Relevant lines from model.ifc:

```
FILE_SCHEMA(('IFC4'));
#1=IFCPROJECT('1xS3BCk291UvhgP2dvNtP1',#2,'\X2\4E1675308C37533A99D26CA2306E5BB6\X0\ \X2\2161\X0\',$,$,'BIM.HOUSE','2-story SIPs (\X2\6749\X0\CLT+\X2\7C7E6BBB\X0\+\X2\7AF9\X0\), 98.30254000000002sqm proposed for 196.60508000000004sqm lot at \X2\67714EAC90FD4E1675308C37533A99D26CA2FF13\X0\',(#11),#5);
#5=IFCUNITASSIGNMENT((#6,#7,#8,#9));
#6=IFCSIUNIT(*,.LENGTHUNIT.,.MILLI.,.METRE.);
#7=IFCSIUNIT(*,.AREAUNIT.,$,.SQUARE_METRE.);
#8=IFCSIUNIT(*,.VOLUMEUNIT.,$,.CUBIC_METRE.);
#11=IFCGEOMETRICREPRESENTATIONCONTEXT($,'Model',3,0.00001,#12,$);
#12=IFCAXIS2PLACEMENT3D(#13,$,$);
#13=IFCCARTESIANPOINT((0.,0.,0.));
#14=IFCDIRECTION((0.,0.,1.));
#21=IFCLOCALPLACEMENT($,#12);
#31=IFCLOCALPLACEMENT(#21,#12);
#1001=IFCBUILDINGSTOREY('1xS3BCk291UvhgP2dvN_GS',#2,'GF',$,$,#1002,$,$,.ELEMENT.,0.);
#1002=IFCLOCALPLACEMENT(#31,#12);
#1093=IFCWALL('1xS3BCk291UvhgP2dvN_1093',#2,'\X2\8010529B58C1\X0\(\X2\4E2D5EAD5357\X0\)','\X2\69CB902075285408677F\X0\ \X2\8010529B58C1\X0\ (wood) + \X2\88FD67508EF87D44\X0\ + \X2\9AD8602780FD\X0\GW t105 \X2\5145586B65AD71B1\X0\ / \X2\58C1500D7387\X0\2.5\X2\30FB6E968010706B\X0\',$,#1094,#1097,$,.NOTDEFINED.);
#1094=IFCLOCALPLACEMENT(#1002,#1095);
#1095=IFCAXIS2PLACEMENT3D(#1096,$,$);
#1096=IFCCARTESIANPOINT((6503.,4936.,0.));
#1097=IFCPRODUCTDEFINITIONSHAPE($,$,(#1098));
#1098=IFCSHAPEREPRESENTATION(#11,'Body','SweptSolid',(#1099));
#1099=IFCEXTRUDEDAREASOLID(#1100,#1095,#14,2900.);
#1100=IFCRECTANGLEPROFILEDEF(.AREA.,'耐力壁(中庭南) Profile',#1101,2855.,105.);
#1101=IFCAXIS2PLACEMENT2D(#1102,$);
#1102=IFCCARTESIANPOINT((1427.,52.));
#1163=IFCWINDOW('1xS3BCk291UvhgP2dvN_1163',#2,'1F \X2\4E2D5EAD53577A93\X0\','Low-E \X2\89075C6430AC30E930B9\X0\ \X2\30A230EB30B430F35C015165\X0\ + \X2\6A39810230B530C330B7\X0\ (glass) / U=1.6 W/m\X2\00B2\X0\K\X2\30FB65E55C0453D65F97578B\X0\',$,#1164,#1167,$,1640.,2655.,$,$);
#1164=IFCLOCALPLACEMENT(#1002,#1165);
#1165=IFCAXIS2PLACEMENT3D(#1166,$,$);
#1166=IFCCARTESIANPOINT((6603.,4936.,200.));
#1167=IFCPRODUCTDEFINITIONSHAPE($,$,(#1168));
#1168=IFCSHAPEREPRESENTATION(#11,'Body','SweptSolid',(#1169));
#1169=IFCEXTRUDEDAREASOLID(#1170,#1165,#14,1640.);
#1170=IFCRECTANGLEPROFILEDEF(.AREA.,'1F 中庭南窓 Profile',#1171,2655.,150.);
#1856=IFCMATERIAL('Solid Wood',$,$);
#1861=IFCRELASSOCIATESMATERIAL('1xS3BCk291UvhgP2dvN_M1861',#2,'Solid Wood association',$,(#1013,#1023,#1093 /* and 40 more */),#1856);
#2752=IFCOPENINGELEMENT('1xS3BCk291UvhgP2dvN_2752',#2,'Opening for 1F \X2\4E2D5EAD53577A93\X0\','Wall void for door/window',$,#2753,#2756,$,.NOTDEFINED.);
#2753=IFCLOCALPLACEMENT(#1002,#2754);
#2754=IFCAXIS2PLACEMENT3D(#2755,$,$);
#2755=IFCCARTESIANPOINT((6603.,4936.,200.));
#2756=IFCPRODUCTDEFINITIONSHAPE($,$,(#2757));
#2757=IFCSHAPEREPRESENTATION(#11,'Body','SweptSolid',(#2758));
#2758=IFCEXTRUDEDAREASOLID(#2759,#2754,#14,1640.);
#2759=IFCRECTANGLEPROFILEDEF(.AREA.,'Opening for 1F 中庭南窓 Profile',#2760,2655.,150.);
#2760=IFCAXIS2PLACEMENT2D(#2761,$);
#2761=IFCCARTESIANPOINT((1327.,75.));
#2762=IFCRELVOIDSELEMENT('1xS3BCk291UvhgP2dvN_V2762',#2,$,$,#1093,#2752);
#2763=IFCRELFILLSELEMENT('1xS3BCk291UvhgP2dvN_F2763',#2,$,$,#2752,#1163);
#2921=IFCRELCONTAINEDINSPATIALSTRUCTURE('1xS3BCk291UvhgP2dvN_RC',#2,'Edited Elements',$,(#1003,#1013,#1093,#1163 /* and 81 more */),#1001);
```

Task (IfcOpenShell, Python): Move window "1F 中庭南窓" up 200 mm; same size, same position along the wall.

```python
import numpy as np
import ifcopenshell
import ifcopenshell.api.geometry
import ifcopenshell.util.placement
import ifcopenshell.util.unit

model = ifcopenshell.open("model.ifc")
unit_scale = ifcopenshell.util.unit.calculate_unit_scale(model)

window = model.by_guid("1xS3BCk291UvhgP2dvN_1163")
opening = window.FillsVoids[0].RelatingOpeningElement
dz = 0.2 / unit_scale

shift = np.array([0.0, 0.0, dz])
# The window is not placed relative to its opening, so move both.
for product in (opening, window):
    matrix = ifcopenshell.util.placement.get_local_placement(product.ObjectPlacement)
    matrix[:3, 3] += shift
    ifcopenshell.api.geometry.edit_object_placement(model, product=product, matrix=matrix, is_si=False)

print(f"moved by {dz * unit_scale:+.3f} m")

model.write("model_v2.ifc")
```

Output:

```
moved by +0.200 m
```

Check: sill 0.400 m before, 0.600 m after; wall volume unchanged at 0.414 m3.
